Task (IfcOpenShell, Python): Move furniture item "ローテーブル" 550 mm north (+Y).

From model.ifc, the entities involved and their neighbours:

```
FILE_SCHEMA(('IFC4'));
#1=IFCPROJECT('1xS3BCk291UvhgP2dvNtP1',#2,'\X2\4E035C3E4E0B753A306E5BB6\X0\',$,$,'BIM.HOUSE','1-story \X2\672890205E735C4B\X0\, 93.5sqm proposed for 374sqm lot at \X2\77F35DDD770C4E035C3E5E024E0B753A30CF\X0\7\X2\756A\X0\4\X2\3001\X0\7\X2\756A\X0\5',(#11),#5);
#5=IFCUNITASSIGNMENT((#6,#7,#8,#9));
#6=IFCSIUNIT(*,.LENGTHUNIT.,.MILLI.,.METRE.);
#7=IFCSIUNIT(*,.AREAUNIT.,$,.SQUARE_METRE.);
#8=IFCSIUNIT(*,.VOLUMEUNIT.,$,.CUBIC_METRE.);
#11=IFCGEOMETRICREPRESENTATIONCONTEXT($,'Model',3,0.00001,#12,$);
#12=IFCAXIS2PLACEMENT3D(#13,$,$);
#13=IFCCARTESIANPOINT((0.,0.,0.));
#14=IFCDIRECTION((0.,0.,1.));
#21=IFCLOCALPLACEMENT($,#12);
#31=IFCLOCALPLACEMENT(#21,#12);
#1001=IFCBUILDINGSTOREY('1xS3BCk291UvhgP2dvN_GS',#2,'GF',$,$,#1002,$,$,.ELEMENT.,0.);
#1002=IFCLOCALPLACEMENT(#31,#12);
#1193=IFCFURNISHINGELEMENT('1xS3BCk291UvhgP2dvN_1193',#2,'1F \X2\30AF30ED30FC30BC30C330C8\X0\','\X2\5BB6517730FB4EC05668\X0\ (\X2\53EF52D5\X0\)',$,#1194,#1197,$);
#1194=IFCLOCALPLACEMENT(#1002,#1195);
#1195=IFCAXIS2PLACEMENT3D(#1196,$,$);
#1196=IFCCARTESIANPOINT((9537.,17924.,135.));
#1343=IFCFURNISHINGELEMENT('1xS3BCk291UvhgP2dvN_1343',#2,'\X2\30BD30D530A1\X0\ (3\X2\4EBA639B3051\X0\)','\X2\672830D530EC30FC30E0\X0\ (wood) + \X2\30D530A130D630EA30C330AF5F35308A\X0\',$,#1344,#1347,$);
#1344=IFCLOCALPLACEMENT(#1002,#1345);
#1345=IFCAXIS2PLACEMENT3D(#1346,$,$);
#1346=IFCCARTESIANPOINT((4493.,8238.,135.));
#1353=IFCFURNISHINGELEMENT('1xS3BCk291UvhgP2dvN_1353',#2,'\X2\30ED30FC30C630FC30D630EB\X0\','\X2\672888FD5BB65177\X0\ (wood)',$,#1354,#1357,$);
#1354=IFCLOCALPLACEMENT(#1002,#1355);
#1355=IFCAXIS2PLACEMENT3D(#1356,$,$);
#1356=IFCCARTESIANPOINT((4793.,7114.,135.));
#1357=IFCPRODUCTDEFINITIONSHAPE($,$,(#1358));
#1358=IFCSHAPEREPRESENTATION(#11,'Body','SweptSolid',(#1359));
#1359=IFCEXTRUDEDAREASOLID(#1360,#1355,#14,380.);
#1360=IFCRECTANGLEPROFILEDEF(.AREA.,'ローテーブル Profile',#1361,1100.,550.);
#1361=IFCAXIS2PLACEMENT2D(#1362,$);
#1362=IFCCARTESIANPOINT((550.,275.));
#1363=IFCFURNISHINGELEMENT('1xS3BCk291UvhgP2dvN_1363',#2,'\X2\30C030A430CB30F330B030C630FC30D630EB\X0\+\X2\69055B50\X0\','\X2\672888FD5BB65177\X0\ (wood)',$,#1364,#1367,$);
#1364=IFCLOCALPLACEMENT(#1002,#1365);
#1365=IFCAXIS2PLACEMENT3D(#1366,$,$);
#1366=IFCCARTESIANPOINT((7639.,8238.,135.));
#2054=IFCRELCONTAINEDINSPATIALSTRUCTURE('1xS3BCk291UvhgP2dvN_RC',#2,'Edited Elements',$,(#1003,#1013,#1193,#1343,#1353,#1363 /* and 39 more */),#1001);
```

```python
import ifcopenshell
import ifcopenshell.api.geometry
import ifcopenshell.util.placement
import ifcopenshell.util.unit

model = ifcopenshell.open("model.ifc")
unit_scale = ifcopenshell.util.unit.calculate_unit_scale(model)

item = model.by_guid("1xS3BCk291UvhgP2dvN_1353")
matrix = ifcopenshell.util.placement.get_local_placement(item.ObjectPlacement)
matrix[1, 3] += 0.55 / unit_scale
ifcopenshell.api.geometry.edit_object_placement(model, product=item, matrix=matrix, is_si=False)

print(ifcopenshell.util.placement.get_local_placement(item.ObjectPlacement).round(3) + 0.0)

model.write("model_updated.ifc")
```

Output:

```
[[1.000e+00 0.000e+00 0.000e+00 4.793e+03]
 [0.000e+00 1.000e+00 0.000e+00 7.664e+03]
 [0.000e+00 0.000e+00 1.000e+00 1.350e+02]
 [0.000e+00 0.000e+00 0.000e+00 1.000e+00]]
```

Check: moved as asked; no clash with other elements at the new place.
